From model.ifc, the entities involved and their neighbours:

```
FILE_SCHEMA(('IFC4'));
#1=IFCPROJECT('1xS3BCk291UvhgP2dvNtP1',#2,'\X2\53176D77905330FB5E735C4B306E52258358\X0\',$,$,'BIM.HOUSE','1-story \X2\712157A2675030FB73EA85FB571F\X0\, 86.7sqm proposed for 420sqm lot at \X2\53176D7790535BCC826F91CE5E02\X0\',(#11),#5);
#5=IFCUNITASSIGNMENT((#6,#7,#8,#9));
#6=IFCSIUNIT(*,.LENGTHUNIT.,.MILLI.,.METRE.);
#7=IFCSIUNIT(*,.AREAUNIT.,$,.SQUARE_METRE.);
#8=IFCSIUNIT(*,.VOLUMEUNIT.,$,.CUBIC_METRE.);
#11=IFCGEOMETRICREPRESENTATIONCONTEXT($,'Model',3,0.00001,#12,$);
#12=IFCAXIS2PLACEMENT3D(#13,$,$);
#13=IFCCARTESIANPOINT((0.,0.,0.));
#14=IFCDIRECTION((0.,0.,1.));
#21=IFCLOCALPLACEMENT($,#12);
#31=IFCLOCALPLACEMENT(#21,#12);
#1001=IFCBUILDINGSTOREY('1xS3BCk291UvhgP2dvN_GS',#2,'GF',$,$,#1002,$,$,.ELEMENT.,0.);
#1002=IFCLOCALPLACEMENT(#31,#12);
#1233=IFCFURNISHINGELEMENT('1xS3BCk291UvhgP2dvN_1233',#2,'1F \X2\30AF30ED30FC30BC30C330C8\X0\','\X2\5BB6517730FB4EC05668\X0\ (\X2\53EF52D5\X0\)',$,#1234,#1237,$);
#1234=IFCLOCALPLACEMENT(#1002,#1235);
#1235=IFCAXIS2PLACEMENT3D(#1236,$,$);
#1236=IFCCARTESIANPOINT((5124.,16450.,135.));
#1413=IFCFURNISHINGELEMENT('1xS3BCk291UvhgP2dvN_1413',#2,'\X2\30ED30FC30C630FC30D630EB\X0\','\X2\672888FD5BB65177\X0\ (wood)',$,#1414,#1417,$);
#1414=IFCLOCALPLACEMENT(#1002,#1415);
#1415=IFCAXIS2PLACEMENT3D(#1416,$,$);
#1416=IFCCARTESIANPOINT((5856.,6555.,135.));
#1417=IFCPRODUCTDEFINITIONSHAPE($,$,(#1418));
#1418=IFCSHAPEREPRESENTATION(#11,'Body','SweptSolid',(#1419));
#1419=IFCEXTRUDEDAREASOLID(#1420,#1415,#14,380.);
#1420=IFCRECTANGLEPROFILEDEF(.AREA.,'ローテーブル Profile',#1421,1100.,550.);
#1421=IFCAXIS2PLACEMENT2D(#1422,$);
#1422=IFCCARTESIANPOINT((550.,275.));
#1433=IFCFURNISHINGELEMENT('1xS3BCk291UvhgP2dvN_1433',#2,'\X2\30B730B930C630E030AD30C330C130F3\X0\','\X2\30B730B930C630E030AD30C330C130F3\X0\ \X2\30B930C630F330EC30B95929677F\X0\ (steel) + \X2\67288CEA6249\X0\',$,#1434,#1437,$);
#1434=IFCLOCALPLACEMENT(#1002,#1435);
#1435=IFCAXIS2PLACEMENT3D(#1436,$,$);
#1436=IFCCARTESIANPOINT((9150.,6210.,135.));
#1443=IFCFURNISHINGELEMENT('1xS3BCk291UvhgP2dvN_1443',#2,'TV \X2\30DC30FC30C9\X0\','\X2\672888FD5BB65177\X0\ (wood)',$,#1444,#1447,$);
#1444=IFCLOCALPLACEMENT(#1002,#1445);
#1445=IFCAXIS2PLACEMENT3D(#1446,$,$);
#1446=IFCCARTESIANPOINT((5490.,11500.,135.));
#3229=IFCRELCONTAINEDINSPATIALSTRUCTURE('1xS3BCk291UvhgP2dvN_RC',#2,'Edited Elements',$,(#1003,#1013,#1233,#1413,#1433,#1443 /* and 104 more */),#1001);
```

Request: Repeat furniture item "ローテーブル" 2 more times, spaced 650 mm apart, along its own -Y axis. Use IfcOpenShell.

```python
import ifcopenshell
import ifcopenshell.api.geometry
import ifcopenshell.api.root
import ifcopenshell.util.element
import ifcopenshell.util.placement
import ifcopenshell.util.unit

model = ifcopenshell.open("model.ifc")
unit_scale = ifcopenshell.util.unit.calculate_unit_scale(model)


def reuse_history(source, copy):
    """copy_class also copies each property set's owner history, people and application; keep the originals."""
    for rel in copy.IsDefinedBy:
        if rel.is_a("IfcRelDefinesByProperties") and (history := rel.RelatingPropertyDefinition.OwnerHistory):
            rel.RelatingPropertyDefinition.OwnerHistory = source.OwnerHistory
            ifcopenshell.util.element.remove_deep2(model, history)


source = model.by_id(1413)
base = ifcopenshell.util.placement.get_local_placement(source.ObjectPlacement)
step = -base[:3, 1] * 0.65 / unit_scale

for i in range(1, 3):
    copy = ifcopenshell.api.root.copy_class(model, product=source)
    copy.Representation = ifcopenshell.util.element.copy_deep(
        model, source.Representation, exclude=["IfcGeometricRepresentationContext", "IfcRepresentationMap"]
    )
    reuse_history(source, copy)
    matrix = base.copy()
    matrix[:3, 3] += i * step
    print("added at", matrix[:3, 3].round(3) + 0.0)
    ifcopenshell.api.geometry.edit_object_placement(model, product=copy, matrix=matrix, is_si=False)

model.write("model_v2.ifc")
```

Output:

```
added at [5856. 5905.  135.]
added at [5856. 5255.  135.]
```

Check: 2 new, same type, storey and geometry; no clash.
